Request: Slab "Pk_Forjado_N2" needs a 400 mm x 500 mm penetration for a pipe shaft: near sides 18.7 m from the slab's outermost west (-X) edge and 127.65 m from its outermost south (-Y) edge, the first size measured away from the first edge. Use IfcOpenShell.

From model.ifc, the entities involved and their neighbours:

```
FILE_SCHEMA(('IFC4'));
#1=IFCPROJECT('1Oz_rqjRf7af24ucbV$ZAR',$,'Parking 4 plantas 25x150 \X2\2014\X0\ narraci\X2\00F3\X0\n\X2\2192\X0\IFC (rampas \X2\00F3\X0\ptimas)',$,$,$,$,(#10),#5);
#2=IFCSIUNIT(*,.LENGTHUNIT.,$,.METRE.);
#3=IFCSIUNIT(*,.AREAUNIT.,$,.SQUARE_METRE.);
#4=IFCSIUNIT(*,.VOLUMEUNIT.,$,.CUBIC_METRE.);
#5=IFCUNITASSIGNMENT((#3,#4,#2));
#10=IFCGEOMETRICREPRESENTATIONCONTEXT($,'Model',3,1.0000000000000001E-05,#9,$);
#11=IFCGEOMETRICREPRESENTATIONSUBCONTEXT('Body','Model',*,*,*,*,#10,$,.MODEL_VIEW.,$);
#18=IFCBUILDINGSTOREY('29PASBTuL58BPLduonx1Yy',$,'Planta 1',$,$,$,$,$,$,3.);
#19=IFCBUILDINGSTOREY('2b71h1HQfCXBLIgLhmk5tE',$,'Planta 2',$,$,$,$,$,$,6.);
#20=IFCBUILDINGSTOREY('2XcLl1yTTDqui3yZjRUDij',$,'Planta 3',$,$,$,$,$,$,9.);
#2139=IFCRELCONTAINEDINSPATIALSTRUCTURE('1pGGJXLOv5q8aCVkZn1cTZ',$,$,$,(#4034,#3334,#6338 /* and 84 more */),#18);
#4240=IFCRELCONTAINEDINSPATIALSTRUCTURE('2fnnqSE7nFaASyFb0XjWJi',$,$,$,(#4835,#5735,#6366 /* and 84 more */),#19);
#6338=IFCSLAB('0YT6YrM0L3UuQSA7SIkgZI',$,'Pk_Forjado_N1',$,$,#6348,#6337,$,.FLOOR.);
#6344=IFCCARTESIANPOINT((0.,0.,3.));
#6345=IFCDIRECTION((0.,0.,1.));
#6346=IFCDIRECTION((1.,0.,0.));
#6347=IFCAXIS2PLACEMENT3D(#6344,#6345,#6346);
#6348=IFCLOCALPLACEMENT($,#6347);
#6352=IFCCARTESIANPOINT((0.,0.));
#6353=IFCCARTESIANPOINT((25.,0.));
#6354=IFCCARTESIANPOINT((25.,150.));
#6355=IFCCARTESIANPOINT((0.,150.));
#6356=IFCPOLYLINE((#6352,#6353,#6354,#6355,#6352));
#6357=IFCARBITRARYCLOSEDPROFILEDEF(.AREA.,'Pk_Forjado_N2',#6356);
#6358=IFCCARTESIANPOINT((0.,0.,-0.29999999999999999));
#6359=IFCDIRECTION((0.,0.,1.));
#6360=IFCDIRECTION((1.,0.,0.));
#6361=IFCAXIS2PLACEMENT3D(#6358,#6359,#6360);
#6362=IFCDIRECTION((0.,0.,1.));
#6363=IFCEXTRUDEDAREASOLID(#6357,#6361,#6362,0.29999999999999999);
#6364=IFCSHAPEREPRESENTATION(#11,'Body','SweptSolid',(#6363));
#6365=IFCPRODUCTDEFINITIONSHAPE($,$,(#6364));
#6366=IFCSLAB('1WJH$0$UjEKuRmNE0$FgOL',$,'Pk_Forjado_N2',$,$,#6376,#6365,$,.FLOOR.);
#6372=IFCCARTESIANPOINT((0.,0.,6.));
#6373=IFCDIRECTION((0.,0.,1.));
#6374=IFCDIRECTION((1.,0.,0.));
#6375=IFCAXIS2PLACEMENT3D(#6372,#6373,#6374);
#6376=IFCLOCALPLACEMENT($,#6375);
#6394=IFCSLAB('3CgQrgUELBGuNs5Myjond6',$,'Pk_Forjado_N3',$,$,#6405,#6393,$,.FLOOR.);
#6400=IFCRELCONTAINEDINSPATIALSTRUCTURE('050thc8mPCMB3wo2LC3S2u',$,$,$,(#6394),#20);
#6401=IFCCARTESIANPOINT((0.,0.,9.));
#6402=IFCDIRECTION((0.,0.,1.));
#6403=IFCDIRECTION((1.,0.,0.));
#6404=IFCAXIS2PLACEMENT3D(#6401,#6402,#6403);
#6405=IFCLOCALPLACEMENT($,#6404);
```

```python
import numpy as np
import ifcopenshell
import ifcopenshell.api.feature
import ifcopenshell.api.geometry
import ifcopenshell.api.root
import ifcopenshell.geom
import ifcopenshell.util.placement
import ifcopenshell.util.representation
import ifcopenshell.util.shape
import ifcopenshell.util.unit

model = ifcopenshell.open("model.ifc")
unit_scale = ifcopenshell.util.unit.calculate_unit_scale(model)
settings = ifcopenshell.geom.settings()


def volume(element):
    """Net volume in cubic metres, openings subtracted."""
    shape = ifcopenshell.geom.create_shape(settings, element)
    return ifcopenshell.util.shape.get_volume(shape.geometry)


slab = model.by_id(6366)
before = volume(slab)

# Extent in the slab's own axes, in metres. The edges named are its -X and -Y sides.
slab_shape = ifcopenshell.geom.create_shape(settings, slab)
vertices = ifcopenshell.util.shape.get_vertices(slab_shape.geometry)
x_min, y_min, bottom = vertices.min(axis=0)
top = vertices[:, 2].max()

opening = ifcopenshell.api.root.create_entity(model, ifc_class="IfcOpeningElement", name="Pipe shaft opening", predefined_type="OPENING")
context = ifcopenshell.util.representation.get_context(model, "Model", "Body", "MODEL_VIEW")
width, depth = 0.4, 0.5
outline = [(0.0, 0.0), (width, 0.0), (width, depth), (0.0, depth), (0.0, 0.0)]
# Overshoot both faces by 50 mm so the cut is clean.
shape = ifcopenshell.api.geometry.add_slab_representation(
    model, context=context, depth=top - bottom + 0.1, polyline=outline
)
ifcopenshell.api.geometry.assign_representation(model, product=opening, representation=shape)

matrix = ifcopenshell.util.placement.get_local_placement(slab.ObjectPlacement)
matrix[:, 3] = matrix @ np.append(np.array([x_min + 18.7, y_min + 127.65, bottom - 0.05]) / unit_scale, 1.0)
ifcopenshell.api.geometry.edit_object_placement(model, product=opening, matrix=matrix, is_si=False)
ifcopenshell.api.feature.add_feature(model, feature=opening, element=slab)

after = volume(slab)

print(f"slab volume {before:.3f} -> {after:.3f} m3")

model.write("model-out.ifc")
```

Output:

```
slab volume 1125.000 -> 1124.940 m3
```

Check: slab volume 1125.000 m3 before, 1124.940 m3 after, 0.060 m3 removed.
